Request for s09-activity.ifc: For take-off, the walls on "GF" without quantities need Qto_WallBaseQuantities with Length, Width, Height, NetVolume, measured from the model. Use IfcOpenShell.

First a look at what the model holds.

```python
import ifcopenshell
import ifcopenshell.util.element
import ifcopenshell.util.unit

model = ifcopenshell.open("s09-activity.ifc")
print(model.schema)
for unit_type in ("LENGTHUNIT", "AREAUNIT", "VOLUMEUNIT"):
    print(unit_type, ifcopenshell.util.unit.calculate_unit_scale(model, unit_type))
storey = next(s for s in model.by_type("IfcBuildingStorey") if s.Name == "GF")
walls = [e for e in ifcopenshell.util.element.get_decomposition(storey) if e.is_a("IfcWall")]
for e in sorted(walls, key=lambda e: e.id()):
    print(e.id(), e.is_a(), e.Name, list(ifcopenshell.util.element.get_psets(e, qtos_only=True)), sep=" | ")
```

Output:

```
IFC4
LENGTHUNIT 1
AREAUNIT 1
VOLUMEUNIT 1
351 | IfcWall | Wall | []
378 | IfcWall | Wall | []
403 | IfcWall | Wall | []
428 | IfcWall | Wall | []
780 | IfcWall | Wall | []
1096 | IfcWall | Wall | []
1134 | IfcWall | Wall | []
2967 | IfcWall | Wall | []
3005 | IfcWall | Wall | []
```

```python
import ifcopenshell
import ifcopenshell.api.pset
import ifcopenshell.geom
import ifcopenshell.util.element
import ifcopenshell.util.shape
import ifcopenshell.util.unit

model = ifcopenshell.open("s09-activity.ifc")
unit_scale = ifcopenshell.util.unit.calculate_unit_scale(model)
volume_scale = ifcopenshell.util.unit.calculate_unit_scale(model, "VOLUMEUNIT")
settings = ifcopenshell.geom.settings()

storey = next(s for s in model.by_type("IfcBuildingStorey") if s.Name == "GF")
walls = [e for e in ifcopenshell.util.element.get_decomposition(storey) if e.is_a("IfcWall")]

for e in sorted(walls, key=lambda e: e.id()):
    if ifcopenshell.util.element.get_psets(e, qtos_only=True, should_inherit=False):
        continue
    # Geometry comes back in metres, in the element's own axes.
    shape = ifcopenshell.geom.create_shape(settings, e)
    values = {
        "Length": ifcopenshell.util.shape.get_x(shape.geometry) / unit_scale,
        "Width": ifcopenshell.util.shape.get_y(shape.geometry) / unit_scale,
        "Height": ifcopenshell.util.shape.get_z(shape.geometry) / unit_scale,
        "NetVolume": ifcopenshell.util.shape.get_volume(shape.geometry) / volume_scale,
    }
    qto = ifcopenshell.api.pset.add_qto(model, product=e, name="Qto_WallBaseQuantities")
    ifcopenshell.api.pset.edit_qto(model, qto=qto, properties=values)
    print(e.id(), {k: round(v, 3) for k, v in values.items()})

model.write("s09-activity_edited.ifc")
```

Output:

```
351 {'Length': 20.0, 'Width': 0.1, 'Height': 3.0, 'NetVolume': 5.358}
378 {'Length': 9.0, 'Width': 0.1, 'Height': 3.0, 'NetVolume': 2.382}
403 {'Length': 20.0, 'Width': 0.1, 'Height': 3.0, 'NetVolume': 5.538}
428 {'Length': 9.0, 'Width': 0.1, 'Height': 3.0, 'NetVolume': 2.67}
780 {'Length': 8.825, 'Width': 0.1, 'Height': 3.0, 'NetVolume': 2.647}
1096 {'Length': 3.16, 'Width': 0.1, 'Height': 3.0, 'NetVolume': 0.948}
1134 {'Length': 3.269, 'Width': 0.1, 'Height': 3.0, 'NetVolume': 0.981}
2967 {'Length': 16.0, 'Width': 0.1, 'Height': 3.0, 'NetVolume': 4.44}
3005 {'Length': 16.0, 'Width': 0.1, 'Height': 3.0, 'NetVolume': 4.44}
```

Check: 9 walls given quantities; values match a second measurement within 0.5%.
